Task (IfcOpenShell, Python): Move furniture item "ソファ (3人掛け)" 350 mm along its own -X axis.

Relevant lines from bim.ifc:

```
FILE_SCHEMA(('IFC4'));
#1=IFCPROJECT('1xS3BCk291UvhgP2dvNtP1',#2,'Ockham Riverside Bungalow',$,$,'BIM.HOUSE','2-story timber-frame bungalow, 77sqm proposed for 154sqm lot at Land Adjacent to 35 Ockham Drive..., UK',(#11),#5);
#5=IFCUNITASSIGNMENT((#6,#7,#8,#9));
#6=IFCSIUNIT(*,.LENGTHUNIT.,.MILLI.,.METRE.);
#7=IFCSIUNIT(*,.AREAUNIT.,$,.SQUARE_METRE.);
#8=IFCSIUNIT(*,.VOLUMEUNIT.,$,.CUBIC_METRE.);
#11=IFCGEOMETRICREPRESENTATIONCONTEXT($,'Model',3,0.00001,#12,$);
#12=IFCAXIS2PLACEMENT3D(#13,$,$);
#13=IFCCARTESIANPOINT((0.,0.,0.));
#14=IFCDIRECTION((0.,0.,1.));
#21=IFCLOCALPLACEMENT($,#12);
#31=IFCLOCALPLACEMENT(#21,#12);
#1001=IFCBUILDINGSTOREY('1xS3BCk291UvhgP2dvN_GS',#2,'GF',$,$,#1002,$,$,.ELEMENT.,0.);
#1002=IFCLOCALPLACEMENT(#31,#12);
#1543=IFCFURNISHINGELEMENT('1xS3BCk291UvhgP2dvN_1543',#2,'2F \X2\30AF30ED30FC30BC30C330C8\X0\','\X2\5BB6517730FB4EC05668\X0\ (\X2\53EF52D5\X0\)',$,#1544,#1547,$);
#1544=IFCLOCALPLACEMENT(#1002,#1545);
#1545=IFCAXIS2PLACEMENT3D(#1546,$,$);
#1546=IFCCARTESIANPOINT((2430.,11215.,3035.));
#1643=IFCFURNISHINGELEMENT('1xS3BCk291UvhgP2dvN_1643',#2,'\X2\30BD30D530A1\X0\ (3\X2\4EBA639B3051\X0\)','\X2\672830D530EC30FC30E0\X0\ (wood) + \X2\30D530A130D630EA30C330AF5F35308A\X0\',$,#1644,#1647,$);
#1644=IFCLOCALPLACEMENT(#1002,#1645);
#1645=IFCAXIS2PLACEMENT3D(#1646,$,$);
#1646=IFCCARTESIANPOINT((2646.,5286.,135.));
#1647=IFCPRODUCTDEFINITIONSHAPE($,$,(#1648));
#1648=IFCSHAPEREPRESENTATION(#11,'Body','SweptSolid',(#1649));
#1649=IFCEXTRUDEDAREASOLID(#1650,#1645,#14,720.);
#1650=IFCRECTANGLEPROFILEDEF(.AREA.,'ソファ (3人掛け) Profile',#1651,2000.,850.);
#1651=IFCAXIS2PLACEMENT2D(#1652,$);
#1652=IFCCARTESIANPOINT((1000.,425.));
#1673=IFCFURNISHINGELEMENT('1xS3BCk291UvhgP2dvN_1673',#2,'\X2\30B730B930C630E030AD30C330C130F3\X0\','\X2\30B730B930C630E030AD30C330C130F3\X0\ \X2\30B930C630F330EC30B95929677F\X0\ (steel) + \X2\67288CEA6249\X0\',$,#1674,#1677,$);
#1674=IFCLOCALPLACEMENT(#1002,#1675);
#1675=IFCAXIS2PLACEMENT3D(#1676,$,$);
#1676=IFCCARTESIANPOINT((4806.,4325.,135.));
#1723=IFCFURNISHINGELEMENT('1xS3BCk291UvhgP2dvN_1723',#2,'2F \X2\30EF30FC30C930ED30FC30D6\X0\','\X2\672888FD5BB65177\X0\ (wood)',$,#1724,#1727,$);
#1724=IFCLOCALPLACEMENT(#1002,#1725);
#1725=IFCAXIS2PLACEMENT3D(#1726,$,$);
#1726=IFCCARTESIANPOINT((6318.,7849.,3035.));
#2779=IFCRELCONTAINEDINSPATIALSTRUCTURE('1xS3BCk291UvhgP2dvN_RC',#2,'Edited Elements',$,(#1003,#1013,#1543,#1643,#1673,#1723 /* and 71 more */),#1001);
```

```python
import ifcopenshell
import ifcopenshell.api.geometry
import ifcopenshell.util.placement

model = ifcopenshell.open("bim.ifc")

item = model.by_id(1643)
matrix = ifcopenshell.util.placement.get_local_placement(item.ObjectPlacement)
matrix[:3, 3] -= matrix[:3, 0] * 350.0
ifcopenshell.api.geometry.edit_object_placement(model, product=item, matrix=matrix, is_si=False)

print(ifcopenshell.util.placement.get_local_placement(item.ObjectPlacement).round(3) + 0.0)

model.write("bim_rev.ifc")
```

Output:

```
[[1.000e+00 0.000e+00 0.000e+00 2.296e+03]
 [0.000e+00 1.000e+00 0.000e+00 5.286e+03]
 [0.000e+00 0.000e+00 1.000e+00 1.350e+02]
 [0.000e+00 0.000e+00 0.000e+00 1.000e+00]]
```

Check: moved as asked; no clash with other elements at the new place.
